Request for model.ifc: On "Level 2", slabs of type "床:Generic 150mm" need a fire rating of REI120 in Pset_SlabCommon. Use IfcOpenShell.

First a look at what the model holds.

```python
import ifcopenshell
import ifcopenshell.util.element

model = ifcopenshell.open("model.ifc")
print(model.schema)
storey = next(s for s in model.by_type("IfcBuildingStorey") if s.Name == "Level 2")
slabs = [e for e in ifcopenshell.util.element.get_decomposition(storey) if e.is_a("IfcSlab")]
seen = {}
for e in slabs:
    element_type = ifcopenshell.util.element.get_type(e)
    key = (element_type.Name if element_type != e and element_type else None, ifcopenshell.util.element.get_pset(e, "Pset_SlabCommon", "FireRating"))
    seen[key] = seen.get(key, 0) + 1
for (name, value), count in sorted(seen.items(), key=str):
    print(count, "x", name, "|", value)
```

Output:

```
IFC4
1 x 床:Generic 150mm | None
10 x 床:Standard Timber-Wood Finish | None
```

```python
import ifcopenshell
import ifcopenshell.api.pset
import ifcopenshell.util.element

model = ifcopenshell.open("model.ifc")

storey = next(s for s in model.by_type("IfcBuildingStorey") if s.Name == "Level 2")
slabs = [e for e in ifcopenshell.util.element.get_decomposition(storey) if e.is_a("IfcSlab")]

count = 0
for e in slabs:
    element_type = ifcopenshell.util.element.get_type(e)
    if element_type in (None, e) or element_type.Name != "床:Generic 150mm":
        continue
    # add_pset returns the element's existing set when there is one.
    pset = ifcopenshell.api.pset.add_pset(model, product=e, name="Pset_SlabCommon")
    ifcopenshell.api.pset.edit_pset(model, pset=pset, properties={"FireRating": "REI120"})
    count += 1

print(count, "slabs updated")

model.write("model_rev.ifc")
```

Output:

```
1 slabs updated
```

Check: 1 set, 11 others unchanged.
